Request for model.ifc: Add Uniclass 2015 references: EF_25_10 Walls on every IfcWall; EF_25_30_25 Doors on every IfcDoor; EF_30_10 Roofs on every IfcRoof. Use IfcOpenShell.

First a look at what the model holds.

```python
import ifcopenshell

model = ifcopenshell.open("model.ifc")
print(model.schema)
print("classifications:", [c.Name for c in model.by_type("IfcClassification")])
for ifc_class in ("IfcDoor", "IfcRoof", "IfcStair", "IfcWall", "IfcWindow"):
    print(ifc_class, len(model.by_type(ifc_class)))
```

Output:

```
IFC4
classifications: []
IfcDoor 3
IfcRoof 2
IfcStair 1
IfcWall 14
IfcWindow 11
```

```python
import ifcopenshell
import ifcopenshell.api.classification

model = ifcopenshell.open("model.ifc")

system = ifcopenshell.api.classification.add_classification(model, classification="Uniclass 2015")

codes = {
    "IfcWall": ("EF_25_10", "Walls"),
    "IfcDoor": ("EF_25_30_25", "Doors"),
    "IfcRoof": ("EF_30_10", "Roofs"),
}
for ifc_class, (code, name) in codes.items():
    products = model.by_type(ifc_class)
    ifcopenshell.api.classification.add_reference(
        model, products=products, classification=system, identification=code, name=name
    )
    print(code, len(products))

model.write("model_edited.ifc")
```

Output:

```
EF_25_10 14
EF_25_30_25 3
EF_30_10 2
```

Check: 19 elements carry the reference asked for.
